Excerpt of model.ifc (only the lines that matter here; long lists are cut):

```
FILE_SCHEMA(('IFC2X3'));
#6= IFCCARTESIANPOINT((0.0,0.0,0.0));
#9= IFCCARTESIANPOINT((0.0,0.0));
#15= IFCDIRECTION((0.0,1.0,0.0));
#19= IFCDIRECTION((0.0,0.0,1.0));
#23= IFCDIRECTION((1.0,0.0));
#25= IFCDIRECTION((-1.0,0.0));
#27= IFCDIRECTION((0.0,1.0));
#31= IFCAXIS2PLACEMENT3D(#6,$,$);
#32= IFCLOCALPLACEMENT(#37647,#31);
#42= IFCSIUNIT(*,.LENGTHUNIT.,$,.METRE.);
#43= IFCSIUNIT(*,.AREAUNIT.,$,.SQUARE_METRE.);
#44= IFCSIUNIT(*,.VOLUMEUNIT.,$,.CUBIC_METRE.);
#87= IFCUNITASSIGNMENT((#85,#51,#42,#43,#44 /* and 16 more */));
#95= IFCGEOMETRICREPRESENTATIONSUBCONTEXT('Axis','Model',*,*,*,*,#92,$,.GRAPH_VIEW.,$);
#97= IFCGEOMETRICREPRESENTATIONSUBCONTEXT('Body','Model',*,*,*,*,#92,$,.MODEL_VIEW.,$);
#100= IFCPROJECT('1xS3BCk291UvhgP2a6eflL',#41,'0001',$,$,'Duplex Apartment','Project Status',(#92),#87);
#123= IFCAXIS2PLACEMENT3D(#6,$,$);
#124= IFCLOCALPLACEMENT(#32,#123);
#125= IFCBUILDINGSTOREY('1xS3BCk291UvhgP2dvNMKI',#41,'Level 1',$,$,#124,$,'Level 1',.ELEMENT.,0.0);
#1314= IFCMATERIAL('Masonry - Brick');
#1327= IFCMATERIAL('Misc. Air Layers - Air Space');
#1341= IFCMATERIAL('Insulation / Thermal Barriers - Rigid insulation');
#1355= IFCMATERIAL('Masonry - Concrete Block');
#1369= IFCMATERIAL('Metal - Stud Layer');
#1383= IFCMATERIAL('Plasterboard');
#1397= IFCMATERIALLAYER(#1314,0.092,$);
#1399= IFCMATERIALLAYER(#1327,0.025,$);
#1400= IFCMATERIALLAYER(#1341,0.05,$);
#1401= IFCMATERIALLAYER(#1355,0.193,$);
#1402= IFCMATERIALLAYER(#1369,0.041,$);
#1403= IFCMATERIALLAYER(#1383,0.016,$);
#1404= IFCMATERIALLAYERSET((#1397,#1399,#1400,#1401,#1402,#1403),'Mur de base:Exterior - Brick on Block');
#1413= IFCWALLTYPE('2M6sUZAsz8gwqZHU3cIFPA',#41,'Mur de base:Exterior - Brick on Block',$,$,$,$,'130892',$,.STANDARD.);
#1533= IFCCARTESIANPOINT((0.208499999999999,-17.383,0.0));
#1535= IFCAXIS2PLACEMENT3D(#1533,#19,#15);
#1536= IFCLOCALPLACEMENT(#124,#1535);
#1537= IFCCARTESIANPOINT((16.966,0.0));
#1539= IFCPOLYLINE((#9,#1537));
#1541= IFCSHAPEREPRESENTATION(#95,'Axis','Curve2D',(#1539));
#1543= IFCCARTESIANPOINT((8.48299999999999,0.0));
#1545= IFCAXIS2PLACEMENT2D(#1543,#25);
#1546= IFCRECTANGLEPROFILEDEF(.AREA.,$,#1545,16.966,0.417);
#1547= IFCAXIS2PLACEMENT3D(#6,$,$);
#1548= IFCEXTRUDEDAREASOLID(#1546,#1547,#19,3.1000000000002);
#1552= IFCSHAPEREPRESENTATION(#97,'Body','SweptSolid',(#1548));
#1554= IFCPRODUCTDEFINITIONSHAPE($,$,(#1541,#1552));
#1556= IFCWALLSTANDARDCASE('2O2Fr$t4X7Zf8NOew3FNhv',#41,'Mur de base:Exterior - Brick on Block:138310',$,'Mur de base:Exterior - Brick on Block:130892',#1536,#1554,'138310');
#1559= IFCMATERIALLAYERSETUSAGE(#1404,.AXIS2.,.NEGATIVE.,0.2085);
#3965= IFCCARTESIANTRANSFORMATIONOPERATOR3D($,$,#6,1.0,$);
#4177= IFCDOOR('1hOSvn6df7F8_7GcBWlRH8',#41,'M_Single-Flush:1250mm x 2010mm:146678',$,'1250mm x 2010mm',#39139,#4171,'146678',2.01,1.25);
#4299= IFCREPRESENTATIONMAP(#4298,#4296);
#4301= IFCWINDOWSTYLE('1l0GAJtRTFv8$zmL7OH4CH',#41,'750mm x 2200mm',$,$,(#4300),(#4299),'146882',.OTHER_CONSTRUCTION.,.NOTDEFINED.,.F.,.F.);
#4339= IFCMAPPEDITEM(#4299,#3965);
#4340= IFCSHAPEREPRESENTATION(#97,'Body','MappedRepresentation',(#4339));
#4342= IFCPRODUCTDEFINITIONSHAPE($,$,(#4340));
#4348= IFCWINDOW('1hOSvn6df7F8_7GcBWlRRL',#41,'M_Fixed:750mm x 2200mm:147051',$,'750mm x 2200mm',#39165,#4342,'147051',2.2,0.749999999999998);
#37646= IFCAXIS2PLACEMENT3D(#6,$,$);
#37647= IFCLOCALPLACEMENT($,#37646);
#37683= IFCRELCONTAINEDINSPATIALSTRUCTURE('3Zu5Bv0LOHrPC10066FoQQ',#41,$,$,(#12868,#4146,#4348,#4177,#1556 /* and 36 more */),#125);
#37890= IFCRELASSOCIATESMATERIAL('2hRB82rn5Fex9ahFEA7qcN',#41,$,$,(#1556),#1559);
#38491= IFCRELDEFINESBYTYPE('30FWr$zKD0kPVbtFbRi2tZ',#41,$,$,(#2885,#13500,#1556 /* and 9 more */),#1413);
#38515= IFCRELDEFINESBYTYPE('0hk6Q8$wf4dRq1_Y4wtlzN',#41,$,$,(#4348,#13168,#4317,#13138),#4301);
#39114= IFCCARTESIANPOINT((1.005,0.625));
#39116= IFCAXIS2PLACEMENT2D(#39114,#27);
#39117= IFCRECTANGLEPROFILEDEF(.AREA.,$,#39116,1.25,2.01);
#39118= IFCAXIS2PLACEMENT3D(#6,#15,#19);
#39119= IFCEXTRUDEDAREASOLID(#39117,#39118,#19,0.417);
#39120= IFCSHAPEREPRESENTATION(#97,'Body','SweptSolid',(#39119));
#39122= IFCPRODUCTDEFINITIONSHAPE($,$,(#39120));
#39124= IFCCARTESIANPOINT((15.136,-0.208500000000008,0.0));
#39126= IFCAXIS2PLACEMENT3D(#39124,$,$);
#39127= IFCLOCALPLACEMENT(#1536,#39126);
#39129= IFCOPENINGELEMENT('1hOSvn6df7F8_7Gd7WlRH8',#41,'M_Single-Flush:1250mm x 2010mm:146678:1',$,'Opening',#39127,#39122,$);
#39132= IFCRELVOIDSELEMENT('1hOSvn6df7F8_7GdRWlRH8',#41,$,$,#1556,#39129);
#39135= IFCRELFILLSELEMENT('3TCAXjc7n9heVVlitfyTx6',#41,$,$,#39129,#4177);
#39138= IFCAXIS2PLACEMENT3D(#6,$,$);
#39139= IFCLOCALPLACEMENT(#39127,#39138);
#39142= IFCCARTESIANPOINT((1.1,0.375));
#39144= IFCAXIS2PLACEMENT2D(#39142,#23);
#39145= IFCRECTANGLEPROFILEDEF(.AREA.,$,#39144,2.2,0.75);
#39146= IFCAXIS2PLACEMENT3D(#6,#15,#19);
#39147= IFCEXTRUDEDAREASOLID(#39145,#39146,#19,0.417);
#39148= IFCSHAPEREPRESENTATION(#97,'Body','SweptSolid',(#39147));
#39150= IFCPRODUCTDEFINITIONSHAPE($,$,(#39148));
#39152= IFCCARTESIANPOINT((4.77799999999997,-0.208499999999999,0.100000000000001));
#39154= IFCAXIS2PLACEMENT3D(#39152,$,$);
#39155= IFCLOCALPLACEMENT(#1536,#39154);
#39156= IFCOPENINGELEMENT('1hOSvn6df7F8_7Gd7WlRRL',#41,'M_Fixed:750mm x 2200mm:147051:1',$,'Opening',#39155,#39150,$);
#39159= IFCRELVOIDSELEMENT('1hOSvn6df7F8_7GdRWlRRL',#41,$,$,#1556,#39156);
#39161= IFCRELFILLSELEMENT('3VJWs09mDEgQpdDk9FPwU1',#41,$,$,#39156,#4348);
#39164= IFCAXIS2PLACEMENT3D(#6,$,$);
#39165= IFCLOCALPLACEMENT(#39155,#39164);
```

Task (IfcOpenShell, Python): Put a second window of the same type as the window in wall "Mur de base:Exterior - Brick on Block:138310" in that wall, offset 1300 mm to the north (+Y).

```python
import ifcopenshell
import ifcopenshell.api.feature
import ifcopenshell.api.geometry
import ifcopenshell.api.root
import ifcopenshell.geom
import ifcopenshell.util.element
import ifcopenshell.util.placement
import ifcopenshell.util.shape
import ifcopenshell.util.unit

model = ifcopenshell.open("model.ifc")
unit_scale = ifcopenshell.util.unit.calculate_unit_scale(model)
settings = ifcopenshell.geom.settings()


def volume(element):
    """Net volume in cubic metres, openings subtracted."""
    shape = ifcopenshell.geom.create_shape(settings, element)
    return ifcopenshell.util.shape.get_volume(shape.geometry)


def reuse_history(source, copy):
    """copy_class also copies each property set's owner history, people and application; keep the originals."""
    for rel in copy.IsDefinedBy:
        if rel.is_a("IfcRelDefinesByProperties") and (history := rel.RelatingPropertyDefinition.OwnerHistory):
            rel.RelatingPropertyDefinition.OwnerHistory = source.OwnerHistory
            ifcopenshell.util.element.remove_deep2(model, history)


window = model.by_guid("1hOSvn6df7F8_7GcBWlRRL")
opening = window.FillsVoids[0].RelatingOpeningElement
wall = opening.VoidsElements[0].RelatingBuildingElement
before = volume(wall)
shift = ifcopenshell.util.placement.get_local_placement(wall.ObjectPlacement)[:3, 0] * 1.3 / unit_scale

# copy_class copies the void relationship, type, container and properties, but no geometry.
new_opening = ifcopenshell.api.root.copy_class(model, product=opening)
new_opening.Representation = ifcopenshell.util.element.copy_deep(
    model, opening.Representation, exclude=["IfcGeometricRepresentationContext", "IfcRepresentationMap"]
)
new_opening.Name = "M_Fixed:750mm x 2200mm"
new_window = ifcopenshell.api.root.copy_class(model, product=window)
new_window.Representation = ifcopenshell.util.element.copy_deep(
    model, window.Representation, exclude=["IfcGeometricRepresentationContext", "IfcRepresentationMap"]
)
new_window.Name = "M_Fixed:750mm x 2200mm"
new_window.Tag = None
reuse_history(window, new_window)
fills = ifcopenshell.api.feature.add_filling(model, opening=new_opening, element=new_window)
fills.OwnerHistory = new_window.OwnerHistory  # required in IFC2X3

for old, new in ((opening, new_opening), (window, new_window)):
    matrix = ifcopenshell.util.placement.get_local_placement(old.ObjectPlacement)
    matrix[:3, 3] += shift
    ifcopenshell.api.geometry.edit_object_placement(model, product=new, matrix=matrix, is_si=False)

after = volume(wall)

print(f"wall volume {before:.3f} -> {after:.3f} m3")

model.write("model_edited.ifc")
```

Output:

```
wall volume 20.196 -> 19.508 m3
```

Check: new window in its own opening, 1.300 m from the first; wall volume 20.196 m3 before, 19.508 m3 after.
